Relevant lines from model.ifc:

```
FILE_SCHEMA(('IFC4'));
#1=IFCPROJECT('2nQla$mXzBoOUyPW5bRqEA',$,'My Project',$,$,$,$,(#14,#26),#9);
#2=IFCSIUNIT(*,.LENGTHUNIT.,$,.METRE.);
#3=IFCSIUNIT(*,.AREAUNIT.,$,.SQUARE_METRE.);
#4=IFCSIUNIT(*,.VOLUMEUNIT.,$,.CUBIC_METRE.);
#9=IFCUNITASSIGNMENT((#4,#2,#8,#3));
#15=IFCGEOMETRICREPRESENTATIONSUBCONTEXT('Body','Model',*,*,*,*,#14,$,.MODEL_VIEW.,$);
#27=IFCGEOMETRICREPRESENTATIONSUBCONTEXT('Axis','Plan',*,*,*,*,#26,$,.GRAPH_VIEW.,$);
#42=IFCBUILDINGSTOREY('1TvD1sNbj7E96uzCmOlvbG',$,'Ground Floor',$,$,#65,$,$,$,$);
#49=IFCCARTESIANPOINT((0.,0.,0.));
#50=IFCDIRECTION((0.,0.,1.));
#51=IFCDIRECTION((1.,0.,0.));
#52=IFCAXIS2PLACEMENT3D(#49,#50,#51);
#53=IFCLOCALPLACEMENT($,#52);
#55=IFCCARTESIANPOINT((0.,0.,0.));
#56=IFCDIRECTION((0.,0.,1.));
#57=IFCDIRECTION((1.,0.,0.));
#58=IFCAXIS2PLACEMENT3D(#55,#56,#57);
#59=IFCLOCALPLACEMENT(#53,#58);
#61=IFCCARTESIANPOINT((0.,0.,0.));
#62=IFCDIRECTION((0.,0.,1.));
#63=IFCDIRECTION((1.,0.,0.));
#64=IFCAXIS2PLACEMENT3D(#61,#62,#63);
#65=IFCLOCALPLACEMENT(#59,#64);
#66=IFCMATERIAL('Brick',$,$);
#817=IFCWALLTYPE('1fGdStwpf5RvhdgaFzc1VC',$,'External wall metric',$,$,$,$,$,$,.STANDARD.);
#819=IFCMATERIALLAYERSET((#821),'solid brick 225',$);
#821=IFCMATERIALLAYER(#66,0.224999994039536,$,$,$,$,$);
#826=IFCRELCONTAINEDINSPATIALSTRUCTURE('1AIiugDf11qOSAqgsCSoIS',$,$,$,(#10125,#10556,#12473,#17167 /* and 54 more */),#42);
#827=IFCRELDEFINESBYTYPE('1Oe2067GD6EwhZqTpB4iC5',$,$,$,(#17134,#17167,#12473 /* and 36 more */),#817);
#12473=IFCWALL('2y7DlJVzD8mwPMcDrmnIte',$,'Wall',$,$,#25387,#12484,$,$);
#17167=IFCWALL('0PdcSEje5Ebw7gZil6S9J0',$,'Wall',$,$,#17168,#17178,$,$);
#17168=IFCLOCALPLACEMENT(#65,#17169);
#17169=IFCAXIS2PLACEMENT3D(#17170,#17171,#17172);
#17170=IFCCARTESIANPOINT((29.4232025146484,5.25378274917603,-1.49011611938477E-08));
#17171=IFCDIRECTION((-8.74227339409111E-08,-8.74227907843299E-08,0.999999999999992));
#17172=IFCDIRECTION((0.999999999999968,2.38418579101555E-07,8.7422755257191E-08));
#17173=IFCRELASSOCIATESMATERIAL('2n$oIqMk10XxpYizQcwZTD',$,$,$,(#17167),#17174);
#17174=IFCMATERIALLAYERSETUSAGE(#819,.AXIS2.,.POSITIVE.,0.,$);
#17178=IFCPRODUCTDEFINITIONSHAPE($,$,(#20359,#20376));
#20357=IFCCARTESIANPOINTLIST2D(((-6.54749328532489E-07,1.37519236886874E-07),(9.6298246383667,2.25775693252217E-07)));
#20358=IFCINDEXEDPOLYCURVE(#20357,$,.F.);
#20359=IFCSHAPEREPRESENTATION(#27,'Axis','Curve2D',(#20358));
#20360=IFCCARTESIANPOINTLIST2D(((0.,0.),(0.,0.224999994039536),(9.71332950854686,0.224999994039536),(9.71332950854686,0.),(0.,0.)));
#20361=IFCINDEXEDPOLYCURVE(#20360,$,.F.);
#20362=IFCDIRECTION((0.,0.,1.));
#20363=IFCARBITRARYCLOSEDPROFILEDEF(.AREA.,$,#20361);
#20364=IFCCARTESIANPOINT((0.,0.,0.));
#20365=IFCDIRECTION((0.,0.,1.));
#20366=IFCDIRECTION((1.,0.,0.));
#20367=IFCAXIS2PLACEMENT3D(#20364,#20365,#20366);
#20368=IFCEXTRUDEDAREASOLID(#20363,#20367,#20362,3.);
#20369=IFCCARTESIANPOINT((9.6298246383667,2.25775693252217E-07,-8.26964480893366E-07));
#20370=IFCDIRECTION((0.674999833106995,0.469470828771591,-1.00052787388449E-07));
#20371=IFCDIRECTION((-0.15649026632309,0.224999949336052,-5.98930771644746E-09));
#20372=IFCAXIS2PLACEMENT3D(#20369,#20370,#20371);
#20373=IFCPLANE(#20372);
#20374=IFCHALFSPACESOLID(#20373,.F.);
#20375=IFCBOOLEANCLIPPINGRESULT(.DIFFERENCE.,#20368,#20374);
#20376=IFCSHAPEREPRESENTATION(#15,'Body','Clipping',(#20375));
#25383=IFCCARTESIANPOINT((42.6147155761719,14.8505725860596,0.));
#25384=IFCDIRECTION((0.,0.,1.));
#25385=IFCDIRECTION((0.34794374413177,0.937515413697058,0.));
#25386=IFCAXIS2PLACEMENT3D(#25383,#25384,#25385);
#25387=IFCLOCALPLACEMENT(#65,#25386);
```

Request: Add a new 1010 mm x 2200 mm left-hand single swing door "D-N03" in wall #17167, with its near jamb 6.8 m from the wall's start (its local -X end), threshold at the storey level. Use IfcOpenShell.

```python
import numpy as np
import ifcopenshell
import ifcopenshell.api.feature
import ifcopenshell.api.geometry
import ifcopenshell.api.root
import ifcopenshell.api.spatial
import ifcopenshell.geom
import ifcopenshell.util.element
import ifcopenshell.util.placement
import ifcopenshell.util.representation
import ifcopenshell.util.shape
import ifcopenshell.util.unit

model = ifcopenshell.open("model.ifc")
unit_scale = ifcopenshell.util.unit.calculate_unit_scale(model)
settings = ifcopenshell.geom.settings()


def volume(element):
    """Net volume in cubic metres, openings subtracted."""
    shape = ifcopenshell.geom.create_shape(settings, element)
    return ifcopenshell.util.shape.get_volume(shape.geometry)


wall = model.by_id(17167)
storey = ifcopenshell.util.element.get_container(wall, ifc_class="IfcBuildingStorey")
context = ifcopenshell.util.representation.get_context(model, "Model", "Body", "MODEL_VIEW")
before = volume(wall)

width, height, from_end, sill = 1.01, 2.2, 6.8, 0.0  # metres

# The wall runs along its own X axis, and the end named is its -X end.
wall_shape = ifcopenshell.geom.create_shape(settings, wall)
x, y, z = ifcopenshell.util.shape.get_vertices(wall_shape.geometry).T
start = x.min() + from_end
face, thickness = float(y.min()), float(y.max() - y.min())
wall_matrix = ifcopenshell.util.placement.get_local_placement(wall.ObjectPlacement)
level = ifcopenshell.util.placement.get_local_placement(storey.ObjectPlacement)[2, 3]


def in_wall(x, y):
    """Placement at x, y metres in the wall's axes, at sill height."""
    matrix = wall_matrix.copy()
    matrix[:, 3] = wall_matrix @ np.array([x / unit_scale, y / unit_scale, 0.0, 1.0])
    matrix[2, 3] = level + sill / unit_scale
    return matrix


# Opening: a box that overshoots both wall faces by 50 mm.
opening = ifcopenshell.api.root.create_entity(model, ifc_class="IfcOpeningElement", predefined_type="OPENING")
box = ifcopenshell.api.geometry.add_wall_representation(
    model, context=context, length=width, height=height, thickness=thickness + 0.1
)
ifcopenshell.api.geometry.assign_representation(model, product=opening, representation=box)
ifcopenshell.api.geometry.edit_object_placement(model, product=opening, matrix=in_wall(start, face - 0.05), is_si=False)
ifcopenshell.api.feature.add_feature(model, feature=opening, element=wall)

door = ifcopenshell.api.root.create_entity(model, ifc_class="IfcDoor", name="D-N03", predefined_type="DOOR")
door.OverallWidth, door.OverallHeight = width / unit_scale, height / unit_scale
door.OperationType = "SINGLE_SWING_LEFT"
body = ifcopenshell.api.geometry.add_door_representation(
    model,
    context=context,
    overall_width=door.OverallWidth,
    overall_height=door.OverallHeight,
    operation_type="SINGLE_SWING_LEFT",
    lining_properties={"LiningDepth": thickness / unit_scale, "ThresholdDepth": thickness / unit_scale},
)
ifcopenshell.api.geometry.assign_representation(model, product=door, representation=body)
ifcopenshell.api.spatial.assign_container(model, products=[door], relating_structure=storey)
ifcopenshell.api.feature.add_filling(model, opening=opening, element=door)

# The lining spans the wall, so the door starts at the wall face.
ifcopenshell.api.geometry.edit_object_placement(model, product=door, matrix=in_wall(start, face), is_si=False)

after = volume(wall)

print(f"wall volume {before:.3f} -> {after:.3f} m3")

model.write("model_edited.ifc")
```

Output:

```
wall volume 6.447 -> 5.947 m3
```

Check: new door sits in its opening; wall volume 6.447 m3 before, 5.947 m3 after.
